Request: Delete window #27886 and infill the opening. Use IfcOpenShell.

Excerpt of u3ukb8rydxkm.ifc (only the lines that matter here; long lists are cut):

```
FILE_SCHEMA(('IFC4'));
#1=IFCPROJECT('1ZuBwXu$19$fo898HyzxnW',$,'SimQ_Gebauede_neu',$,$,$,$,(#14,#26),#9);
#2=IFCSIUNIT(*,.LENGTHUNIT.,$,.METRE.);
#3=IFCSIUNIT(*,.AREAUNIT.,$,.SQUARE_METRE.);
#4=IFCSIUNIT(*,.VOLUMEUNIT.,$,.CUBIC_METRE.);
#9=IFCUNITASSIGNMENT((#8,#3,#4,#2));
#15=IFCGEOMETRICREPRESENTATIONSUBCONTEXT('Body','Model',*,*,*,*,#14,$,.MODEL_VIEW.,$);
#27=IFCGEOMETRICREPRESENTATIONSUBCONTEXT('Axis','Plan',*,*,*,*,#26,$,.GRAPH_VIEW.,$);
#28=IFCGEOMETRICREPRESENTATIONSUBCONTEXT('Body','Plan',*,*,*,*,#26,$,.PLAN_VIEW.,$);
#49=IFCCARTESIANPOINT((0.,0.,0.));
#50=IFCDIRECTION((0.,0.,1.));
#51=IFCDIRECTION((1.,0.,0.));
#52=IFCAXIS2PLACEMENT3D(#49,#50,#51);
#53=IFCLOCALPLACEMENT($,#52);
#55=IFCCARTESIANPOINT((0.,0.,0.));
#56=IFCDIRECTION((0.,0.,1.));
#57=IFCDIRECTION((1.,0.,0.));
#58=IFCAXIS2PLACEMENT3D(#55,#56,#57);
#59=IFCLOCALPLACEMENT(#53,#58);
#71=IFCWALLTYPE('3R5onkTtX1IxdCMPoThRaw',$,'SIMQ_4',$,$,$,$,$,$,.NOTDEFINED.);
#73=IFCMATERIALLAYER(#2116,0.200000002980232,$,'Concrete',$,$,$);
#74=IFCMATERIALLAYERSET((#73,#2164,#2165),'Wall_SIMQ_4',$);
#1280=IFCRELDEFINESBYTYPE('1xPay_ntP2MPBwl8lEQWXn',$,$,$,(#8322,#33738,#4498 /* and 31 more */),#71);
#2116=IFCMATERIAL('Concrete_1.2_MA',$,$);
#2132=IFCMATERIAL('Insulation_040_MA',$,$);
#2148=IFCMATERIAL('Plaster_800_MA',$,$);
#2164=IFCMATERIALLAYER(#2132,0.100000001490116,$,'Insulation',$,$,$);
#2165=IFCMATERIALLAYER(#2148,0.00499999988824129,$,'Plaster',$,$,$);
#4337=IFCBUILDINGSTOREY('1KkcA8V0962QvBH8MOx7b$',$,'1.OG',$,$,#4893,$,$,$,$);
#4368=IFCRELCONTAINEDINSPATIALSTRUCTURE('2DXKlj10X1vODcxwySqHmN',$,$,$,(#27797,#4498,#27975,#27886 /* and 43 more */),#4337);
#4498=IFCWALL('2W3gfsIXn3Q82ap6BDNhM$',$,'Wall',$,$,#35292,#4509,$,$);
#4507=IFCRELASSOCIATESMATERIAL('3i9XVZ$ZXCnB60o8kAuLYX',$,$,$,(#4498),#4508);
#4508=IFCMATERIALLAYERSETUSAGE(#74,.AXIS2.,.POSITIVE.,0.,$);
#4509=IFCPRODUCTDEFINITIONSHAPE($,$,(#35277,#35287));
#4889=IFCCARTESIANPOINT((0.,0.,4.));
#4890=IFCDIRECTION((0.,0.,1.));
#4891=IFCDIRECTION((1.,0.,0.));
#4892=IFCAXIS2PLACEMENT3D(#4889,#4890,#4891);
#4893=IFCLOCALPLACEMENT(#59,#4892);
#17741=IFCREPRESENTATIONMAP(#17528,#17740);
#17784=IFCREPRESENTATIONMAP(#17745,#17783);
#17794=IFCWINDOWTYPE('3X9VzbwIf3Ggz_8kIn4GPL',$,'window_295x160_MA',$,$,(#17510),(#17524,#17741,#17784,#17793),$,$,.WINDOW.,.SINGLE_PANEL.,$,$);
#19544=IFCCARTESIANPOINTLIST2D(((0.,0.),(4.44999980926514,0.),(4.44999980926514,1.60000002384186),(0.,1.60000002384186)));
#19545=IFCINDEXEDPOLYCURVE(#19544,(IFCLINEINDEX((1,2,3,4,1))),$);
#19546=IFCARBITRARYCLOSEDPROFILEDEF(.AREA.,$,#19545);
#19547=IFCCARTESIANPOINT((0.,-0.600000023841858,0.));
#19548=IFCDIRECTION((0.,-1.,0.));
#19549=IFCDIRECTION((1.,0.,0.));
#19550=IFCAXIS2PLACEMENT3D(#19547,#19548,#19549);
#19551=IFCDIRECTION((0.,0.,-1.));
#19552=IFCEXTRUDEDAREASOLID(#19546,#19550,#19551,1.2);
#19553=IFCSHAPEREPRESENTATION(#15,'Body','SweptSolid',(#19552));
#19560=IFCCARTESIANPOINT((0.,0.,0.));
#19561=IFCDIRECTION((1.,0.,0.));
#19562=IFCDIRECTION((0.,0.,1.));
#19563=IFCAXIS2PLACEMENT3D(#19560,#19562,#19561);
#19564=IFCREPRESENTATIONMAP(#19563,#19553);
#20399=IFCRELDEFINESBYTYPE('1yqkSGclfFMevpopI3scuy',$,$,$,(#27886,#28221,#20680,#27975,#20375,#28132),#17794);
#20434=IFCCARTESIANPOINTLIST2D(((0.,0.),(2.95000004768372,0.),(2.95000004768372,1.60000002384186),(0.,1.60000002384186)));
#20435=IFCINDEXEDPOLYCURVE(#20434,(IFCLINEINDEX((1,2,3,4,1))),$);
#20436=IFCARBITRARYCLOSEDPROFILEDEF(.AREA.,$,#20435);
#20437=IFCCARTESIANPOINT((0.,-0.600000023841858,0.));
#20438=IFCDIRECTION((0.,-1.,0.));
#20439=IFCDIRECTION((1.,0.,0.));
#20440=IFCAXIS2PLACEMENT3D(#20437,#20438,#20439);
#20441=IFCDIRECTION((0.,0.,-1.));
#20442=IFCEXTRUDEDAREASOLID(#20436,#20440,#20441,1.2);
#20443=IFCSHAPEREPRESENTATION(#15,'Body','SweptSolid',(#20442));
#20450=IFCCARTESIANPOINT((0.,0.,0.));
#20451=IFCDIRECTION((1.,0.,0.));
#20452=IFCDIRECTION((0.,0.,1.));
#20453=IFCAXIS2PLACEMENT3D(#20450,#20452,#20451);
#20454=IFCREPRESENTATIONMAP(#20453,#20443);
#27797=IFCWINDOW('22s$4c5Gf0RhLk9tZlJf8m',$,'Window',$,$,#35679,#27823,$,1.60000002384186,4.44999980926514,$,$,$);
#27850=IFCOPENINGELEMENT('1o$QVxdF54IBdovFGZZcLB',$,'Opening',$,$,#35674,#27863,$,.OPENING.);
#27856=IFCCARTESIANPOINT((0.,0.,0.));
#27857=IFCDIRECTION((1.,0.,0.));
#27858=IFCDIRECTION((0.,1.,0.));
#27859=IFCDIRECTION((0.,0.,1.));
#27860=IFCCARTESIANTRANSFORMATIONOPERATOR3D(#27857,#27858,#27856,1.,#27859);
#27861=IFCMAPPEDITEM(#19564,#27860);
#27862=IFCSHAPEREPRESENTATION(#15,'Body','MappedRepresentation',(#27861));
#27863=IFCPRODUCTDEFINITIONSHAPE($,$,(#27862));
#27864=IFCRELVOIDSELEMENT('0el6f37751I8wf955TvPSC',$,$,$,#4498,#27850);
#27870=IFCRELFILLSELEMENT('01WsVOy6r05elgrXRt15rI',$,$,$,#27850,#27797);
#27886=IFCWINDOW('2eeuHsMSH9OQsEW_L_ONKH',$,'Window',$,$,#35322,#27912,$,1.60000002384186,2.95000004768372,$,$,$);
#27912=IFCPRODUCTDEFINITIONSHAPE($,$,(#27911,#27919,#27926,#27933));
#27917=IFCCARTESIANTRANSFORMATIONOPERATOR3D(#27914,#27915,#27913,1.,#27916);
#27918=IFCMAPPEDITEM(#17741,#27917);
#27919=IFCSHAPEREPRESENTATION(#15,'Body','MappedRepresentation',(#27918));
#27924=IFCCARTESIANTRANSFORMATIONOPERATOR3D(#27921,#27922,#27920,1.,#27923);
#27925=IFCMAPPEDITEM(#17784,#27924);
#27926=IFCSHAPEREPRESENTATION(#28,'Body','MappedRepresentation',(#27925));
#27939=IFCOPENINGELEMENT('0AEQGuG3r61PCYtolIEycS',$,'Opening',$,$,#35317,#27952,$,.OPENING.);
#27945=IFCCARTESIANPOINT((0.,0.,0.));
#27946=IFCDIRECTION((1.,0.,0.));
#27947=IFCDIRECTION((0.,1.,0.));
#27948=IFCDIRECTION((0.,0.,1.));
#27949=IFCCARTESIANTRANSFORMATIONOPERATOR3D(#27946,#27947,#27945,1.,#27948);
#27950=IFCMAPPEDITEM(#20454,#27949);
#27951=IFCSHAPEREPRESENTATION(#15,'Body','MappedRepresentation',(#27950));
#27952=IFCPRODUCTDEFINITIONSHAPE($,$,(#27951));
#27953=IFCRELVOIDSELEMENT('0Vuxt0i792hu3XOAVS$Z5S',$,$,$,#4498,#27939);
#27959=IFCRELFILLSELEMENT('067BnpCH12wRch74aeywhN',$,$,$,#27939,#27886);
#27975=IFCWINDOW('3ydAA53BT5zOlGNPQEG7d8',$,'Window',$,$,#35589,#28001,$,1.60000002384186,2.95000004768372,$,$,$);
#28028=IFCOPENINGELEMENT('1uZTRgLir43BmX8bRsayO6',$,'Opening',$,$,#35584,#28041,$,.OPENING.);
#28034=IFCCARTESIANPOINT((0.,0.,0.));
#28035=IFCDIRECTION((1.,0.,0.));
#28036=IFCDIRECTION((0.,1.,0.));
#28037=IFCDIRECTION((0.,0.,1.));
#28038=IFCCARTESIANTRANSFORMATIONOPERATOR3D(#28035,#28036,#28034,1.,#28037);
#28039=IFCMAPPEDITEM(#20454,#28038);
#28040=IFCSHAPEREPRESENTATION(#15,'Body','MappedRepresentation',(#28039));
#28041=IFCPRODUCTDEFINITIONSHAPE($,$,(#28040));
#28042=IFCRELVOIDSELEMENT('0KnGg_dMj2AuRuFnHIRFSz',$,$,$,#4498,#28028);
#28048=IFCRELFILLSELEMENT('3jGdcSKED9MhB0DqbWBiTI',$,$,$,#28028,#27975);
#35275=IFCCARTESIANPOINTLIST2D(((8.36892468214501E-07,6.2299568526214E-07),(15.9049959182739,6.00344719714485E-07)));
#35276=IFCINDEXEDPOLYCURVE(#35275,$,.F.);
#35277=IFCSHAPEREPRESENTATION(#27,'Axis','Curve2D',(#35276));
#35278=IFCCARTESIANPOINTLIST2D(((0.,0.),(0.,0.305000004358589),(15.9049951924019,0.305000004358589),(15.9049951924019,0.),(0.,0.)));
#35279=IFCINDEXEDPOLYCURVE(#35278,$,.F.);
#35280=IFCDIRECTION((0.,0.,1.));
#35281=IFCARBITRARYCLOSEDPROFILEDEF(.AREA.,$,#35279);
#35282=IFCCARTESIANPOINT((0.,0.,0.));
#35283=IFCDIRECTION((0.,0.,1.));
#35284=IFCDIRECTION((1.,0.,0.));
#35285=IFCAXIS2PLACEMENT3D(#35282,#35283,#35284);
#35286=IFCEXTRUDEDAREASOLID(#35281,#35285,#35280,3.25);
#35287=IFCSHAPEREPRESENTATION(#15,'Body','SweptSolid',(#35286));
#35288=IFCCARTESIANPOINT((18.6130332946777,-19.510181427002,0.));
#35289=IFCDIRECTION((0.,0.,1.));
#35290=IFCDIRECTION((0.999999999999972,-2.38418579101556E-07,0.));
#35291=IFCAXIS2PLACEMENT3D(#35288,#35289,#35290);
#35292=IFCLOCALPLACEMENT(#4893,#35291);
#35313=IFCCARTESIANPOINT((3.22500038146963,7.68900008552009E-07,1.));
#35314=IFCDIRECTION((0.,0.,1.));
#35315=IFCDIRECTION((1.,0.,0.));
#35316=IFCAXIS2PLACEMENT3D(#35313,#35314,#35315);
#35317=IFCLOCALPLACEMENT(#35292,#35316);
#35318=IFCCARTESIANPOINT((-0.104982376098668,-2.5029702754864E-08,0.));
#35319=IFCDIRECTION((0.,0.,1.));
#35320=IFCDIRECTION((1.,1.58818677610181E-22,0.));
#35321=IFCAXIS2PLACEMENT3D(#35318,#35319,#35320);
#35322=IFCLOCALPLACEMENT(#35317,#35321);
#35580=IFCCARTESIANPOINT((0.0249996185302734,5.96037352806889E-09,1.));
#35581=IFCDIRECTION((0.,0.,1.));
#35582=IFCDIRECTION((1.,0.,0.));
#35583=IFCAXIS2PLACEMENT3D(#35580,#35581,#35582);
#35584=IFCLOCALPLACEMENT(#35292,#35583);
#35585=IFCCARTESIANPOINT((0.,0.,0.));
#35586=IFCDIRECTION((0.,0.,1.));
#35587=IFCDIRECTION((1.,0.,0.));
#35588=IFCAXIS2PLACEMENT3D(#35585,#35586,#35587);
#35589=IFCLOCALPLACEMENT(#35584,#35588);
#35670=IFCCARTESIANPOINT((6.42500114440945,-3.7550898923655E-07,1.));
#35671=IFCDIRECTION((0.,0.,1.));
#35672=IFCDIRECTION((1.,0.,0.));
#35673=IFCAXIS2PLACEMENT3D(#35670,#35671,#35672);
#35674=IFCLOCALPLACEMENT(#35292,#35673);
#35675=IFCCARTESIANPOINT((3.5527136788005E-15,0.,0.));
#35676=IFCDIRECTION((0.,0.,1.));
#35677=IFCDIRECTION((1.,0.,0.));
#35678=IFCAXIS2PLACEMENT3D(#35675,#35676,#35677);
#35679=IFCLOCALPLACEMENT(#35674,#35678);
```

```python
import ifcopenshell
import ifcopenshell.api.feature
import ifcopenshell.api.root
import ifcopenshell.geom
import ifcopenshell.util.shape

model = ifcopenshell.open("u3ukb8rydxkm.ifc")
settings = ifcopenshell.geom.settings()


def volume(element):
    """Net volume in cubic metres, openings subtracted."""
    shape = ifcopenshell.geom.create_shape(settings, element)
    return ifcopenshell.util.shape.get_volume(shape.geometry)


window = model.by_guid("2eeuHsMSH9OQsEW_L_ONKH")
opening = window.FillsVoids[0].RelatingOpeningElement
wall = opening.VoidsElements[0].RelatingBuildingElement
before = volume(wall)

ifcopenshell.api.root.remove_product(model, product=window)
ifcopenshell.api.feature.remove_feature(model, feature=opening)

after = volume(wall)

print(f"wall volume {before:.3f} -> {after:.3f} m3")

model.write("u3ukb8rydxkm_v2.ifc")
```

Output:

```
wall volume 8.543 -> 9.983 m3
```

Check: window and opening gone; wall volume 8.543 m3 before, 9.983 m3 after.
